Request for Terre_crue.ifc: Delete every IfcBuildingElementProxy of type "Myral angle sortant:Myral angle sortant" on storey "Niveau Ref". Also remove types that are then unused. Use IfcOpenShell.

First a look at what the model holds.

```python
import ifcopenshell
import ifcopenshell.util.element

model = ifcopenshell.open("Terre_crue.ifc")
print(model.schema)
storey = next(s for s in model.by_type("IfcBuildingStorey") if s.Name == "Niveau Ref")
proxies = [e for e in ifcopenshell.util.element.get_decomposition(storey) if e.is_a("IfcBuildingElementProxy")]
seen = {}
for e in proxies:
    element_type = ifcopenshell.util.element.get_type(e)
    name = element_type.Name if element_type not in (None, e) else None
    seen[name] = seen.get(name, 0) + 1
for name, count in sorted(seen.items(), key=str):
    print(count, "x", name)
```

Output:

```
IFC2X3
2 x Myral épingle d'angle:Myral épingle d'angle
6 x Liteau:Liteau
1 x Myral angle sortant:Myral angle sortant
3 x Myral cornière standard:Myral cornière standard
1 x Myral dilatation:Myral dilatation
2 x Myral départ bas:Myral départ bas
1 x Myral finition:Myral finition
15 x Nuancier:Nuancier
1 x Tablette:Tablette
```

```python
import ifcopenshell
import ifcopenshell.api.root
import ifcopenshell.util.element

model = ifcopenshell.open("Terre_crue.ifc")

storey = next(s for s in model.by_type("IfcBuildingStorey") if s.Name == "Niveau Ref")
proxies = [e for e in ifcopenshell.util.element.get_decomposition(storey) if e.is_a("IfcBuildingElementProxy")]
targets = [e for e in proxies if (t := ifcopenshell.util.element.get_type(e)) not in (None, e) and t.Name == "Myral angle sortant:Myral angle sortant"]
types = {ifcopenshell.util.element.get_type(e) for e in targets} - {None, *targets}

for e in targets:
    ifcopenshell.api.root.remove_product(model, product=e)
print(len(targets), "removed")

unused = [t for t in types if not ifcopenshell.util.element.get_types(t)]
for t in unused:
    ifcopenshell.api.root.remove_product(model, product=t)
print(len(unused), "unused types removed")

model.write("Terre_crue_updated.ifc")
```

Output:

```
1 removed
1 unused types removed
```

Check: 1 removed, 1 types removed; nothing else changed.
